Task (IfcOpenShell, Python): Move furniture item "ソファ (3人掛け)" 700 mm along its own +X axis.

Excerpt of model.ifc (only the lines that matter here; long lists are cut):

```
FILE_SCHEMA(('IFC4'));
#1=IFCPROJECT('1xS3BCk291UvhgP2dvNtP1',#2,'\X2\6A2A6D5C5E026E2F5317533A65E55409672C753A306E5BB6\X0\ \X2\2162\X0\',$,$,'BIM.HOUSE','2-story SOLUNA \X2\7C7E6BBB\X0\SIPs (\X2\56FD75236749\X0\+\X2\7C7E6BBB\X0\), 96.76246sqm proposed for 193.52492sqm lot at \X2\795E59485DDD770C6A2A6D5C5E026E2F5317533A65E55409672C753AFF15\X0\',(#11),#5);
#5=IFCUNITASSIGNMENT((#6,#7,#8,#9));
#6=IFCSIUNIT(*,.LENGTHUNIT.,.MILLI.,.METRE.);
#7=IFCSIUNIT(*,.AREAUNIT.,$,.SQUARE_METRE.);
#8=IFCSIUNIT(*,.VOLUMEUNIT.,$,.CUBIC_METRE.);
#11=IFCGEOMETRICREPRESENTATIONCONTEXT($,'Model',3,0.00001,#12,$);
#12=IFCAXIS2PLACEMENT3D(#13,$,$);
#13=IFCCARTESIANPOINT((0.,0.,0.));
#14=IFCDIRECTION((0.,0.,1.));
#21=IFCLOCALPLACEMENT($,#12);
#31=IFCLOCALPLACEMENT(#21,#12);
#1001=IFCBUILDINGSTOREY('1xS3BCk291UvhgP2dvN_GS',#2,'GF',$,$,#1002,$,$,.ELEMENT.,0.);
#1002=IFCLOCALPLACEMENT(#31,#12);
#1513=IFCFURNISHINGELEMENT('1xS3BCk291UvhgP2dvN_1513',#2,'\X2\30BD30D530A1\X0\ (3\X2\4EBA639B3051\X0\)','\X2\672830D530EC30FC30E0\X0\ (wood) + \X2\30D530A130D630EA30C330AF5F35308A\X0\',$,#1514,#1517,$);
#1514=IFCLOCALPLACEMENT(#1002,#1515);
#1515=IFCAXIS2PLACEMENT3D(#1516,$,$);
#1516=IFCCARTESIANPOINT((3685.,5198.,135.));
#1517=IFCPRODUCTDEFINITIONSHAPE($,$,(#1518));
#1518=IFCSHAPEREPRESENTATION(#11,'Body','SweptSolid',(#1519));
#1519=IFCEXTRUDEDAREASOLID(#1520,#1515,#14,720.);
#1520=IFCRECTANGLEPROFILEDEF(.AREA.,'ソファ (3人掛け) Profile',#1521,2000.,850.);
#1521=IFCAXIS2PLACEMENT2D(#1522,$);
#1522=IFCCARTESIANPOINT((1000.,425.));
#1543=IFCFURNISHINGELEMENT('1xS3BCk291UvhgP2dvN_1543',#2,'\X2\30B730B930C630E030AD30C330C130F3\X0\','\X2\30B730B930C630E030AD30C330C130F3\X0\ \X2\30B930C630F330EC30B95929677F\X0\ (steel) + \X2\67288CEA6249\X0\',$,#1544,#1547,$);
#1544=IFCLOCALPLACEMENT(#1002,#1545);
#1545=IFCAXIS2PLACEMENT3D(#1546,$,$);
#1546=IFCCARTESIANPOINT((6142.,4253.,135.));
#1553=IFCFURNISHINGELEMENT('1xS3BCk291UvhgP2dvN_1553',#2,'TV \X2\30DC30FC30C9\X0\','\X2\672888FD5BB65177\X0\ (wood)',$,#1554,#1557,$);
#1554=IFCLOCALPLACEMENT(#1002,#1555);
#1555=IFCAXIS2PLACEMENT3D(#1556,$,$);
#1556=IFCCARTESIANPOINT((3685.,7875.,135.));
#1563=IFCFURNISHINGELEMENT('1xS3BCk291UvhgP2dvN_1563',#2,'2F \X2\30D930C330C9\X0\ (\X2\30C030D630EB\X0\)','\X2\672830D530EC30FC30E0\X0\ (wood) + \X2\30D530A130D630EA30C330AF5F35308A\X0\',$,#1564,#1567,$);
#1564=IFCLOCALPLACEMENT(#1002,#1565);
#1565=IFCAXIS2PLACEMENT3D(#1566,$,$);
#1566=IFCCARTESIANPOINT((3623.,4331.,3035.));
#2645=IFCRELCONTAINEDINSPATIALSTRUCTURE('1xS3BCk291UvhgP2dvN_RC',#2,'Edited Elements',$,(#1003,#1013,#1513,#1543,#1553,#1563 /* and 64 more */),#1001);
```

```python
import ifcopenshell
import ifcopenshell.api.geometry
import ifcopenshell.util.placement

model = ifcopenshell.open("model.ifc")

item = model.by_id(1513)
matrix = ifcopenshell.util.placement.get_local_placement(item.ObjectPlacement)
matrix[:3, 3] += matrix[:3, 0] * 700.0
ifcopenshell.api.geometry.edit_object_placement(model, product=item, matrix=matrix, is_si=False)

print(ifcopenshell.util.placement.get_local_placement(item.ObjectPlacement).round(3) + 0.0)

model.write("model_edited.ifc")
```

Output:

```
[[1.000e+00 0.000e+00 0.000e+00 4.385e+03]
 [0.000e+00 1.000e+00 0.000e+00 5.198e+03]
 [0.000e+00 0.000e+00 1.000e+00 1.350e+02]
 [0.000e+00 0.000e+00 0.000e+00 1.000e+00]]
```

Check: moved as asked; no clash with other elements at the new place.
